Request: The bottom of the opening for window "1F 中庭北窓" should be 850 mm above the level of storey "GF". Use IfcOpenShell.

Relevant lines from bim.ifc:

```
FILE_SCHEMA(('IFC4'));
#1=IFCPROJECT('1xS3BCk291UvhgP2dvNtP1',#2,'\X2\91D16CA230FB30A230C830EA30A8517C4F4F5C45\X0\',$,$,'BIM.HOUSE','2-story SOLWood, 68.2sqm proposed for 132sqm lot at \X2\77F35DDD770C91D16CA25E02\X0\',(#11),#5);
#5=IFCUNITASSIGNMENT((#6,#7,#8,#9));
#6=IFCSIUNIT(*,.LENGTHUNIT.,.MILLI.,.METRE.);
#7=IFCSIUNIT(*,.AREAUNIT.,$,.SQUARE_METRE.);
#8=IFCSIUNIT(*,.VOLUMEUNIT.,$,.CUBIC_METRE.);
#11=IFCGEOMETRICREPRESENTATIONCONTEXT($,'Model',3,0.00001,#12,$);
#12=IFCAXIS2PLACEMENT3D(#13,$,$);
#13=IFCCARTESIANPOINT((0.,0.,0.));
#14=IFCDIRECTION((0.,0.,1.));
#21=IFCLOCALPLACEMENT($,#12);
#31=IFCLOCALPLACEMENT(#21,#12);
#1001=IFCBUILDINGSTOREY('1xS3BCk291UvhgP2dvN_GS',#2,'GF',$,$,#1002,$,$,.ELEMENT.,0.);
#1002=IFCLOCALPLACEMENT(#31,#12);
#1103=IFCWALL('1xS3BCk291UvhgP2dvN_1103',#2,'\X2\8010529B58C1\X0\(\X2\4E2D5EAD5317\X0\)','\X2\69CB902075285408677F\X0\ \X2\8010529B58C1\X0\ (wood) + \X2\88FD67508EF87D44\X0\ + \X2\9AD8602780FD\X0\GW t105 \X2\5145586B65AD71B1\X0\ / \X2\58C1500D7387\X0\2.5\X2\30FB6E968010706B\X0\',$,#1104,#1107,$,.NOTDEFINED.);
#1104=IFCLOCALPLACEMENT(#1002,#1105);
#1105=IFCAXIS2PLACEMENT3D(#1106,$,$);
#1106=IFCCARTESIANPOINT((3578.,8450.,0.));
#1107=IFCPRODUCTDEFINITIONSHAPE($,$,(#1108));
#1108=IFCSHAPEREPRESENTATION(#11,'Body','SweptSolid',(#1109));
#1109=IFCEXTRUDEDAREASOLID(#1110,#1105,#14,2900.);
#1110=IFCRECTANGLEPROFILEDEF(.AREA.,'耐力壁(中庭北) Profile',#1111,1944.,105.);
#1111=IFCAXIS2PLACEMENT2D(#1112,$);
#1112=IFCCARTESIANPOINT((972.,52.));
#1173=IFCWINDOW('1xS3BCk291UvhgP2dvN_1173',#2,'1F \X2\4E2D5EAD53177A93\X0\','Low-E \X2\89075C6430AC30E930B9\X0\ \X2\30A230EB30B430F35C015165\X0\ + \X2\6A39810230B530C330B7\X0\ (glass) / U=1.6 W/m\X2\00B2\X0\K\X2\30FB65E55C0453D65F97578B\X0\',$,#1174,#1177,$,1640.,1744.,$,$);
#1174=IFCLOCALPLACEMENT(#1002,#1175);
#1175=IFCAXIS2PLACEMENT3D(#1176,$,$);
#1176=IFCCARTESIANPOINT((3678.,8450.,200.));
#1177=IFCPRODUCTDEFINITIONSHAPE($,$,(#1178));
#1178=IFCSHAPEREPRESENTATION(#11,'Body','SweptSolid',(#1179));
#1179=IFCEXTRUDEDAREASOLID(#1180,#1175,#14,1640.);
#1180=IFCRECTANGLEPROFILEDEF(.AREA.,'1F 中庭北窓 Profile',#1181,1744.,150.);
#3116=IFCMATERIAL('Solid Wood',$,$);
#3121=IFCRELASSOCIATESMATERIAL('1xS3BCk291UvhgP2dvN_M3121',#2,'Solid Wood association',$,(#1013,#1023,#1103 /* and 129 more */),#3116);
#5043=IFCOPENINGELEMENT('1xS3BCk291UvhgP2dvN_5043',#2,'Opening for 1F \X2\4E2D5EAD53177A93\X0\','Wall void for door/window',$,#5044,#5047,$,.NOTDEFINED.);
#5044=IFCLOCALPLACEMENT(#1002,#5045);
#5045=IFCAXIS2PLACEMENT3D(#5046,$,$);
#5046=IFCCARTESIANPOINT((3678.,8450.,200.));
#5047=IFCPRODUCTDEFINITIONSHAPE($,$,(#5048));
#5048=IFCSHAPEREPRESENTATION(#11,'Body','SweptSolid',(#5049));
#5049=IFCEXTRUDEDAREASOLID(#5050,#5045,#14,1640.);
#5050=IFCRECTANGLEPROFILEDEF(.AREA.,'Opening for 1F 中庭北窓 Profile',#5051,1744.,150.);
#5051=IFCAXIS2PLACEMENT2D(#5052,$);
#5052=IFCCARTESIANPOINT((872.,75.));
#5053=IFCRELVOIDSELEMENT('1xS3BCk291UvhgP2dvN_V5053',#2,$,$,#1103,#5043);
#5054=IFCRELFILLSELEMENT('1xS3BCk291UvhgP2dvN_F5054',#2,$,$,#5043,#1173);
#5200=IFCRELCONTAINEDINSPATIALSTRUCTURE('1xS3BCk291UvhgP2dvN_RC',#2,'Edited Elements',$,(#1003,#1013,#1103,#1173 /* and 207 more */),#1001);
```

```python
import numpy as np
import ifcopenshell
import ifcopenshell.api.geometry
import ifcopenshell.geom
import ifcopenshell.util.element
import ifcopenshell.util.placement
import ifcopenshell.util.shape
import ifcopenshell.util.unit

model = ifcopenshell.open("bim.ifc")
unit_scale = ifcopenshell.util.unit.calculate_unit_scale(model)

window = model.by_id(1173)
opening = window.FillsVoids[0].RelatingOpeningElement
storey = ifcopenshell.util.element.get_container(window, ifc_class="IfcBuildingStorey")
level = ifcopenshell.util.placement.get_local_placement(storey.ObjectPlacement)[2, 3]

# The opening's origin need not be at the sill, so measure its lowest point.
shape = ifcopenshell.geom.create_shape(ifcopenshell.geom.settings(), opening)
bottom = ifcopenshell.util.shape.get_shape_bottom_elevation(shape, shape.geometry) / unit_scale
dz = level + 0.85 / unit_scale - bottom

shift = np.array([0.0, 0.0, dz])
# The window is not placed relative to its opening, so move both.
for product in (opening, window):
    matrix = ifcopenshell.util.placement.get_local_placement(product.ObjectPlacement)
    matrix[:3, 3] += shift
    ifcopenshell.api.geometry.edit_object_placement(model, product=product, matrix=matrix, is_si=False)

print(f"moved by {dz * unit_scale:+.3f} m")

model.write("bim_edited.ifc")
```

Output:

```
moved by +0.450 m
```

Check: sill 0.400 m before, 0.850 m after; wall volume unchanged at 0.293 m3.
